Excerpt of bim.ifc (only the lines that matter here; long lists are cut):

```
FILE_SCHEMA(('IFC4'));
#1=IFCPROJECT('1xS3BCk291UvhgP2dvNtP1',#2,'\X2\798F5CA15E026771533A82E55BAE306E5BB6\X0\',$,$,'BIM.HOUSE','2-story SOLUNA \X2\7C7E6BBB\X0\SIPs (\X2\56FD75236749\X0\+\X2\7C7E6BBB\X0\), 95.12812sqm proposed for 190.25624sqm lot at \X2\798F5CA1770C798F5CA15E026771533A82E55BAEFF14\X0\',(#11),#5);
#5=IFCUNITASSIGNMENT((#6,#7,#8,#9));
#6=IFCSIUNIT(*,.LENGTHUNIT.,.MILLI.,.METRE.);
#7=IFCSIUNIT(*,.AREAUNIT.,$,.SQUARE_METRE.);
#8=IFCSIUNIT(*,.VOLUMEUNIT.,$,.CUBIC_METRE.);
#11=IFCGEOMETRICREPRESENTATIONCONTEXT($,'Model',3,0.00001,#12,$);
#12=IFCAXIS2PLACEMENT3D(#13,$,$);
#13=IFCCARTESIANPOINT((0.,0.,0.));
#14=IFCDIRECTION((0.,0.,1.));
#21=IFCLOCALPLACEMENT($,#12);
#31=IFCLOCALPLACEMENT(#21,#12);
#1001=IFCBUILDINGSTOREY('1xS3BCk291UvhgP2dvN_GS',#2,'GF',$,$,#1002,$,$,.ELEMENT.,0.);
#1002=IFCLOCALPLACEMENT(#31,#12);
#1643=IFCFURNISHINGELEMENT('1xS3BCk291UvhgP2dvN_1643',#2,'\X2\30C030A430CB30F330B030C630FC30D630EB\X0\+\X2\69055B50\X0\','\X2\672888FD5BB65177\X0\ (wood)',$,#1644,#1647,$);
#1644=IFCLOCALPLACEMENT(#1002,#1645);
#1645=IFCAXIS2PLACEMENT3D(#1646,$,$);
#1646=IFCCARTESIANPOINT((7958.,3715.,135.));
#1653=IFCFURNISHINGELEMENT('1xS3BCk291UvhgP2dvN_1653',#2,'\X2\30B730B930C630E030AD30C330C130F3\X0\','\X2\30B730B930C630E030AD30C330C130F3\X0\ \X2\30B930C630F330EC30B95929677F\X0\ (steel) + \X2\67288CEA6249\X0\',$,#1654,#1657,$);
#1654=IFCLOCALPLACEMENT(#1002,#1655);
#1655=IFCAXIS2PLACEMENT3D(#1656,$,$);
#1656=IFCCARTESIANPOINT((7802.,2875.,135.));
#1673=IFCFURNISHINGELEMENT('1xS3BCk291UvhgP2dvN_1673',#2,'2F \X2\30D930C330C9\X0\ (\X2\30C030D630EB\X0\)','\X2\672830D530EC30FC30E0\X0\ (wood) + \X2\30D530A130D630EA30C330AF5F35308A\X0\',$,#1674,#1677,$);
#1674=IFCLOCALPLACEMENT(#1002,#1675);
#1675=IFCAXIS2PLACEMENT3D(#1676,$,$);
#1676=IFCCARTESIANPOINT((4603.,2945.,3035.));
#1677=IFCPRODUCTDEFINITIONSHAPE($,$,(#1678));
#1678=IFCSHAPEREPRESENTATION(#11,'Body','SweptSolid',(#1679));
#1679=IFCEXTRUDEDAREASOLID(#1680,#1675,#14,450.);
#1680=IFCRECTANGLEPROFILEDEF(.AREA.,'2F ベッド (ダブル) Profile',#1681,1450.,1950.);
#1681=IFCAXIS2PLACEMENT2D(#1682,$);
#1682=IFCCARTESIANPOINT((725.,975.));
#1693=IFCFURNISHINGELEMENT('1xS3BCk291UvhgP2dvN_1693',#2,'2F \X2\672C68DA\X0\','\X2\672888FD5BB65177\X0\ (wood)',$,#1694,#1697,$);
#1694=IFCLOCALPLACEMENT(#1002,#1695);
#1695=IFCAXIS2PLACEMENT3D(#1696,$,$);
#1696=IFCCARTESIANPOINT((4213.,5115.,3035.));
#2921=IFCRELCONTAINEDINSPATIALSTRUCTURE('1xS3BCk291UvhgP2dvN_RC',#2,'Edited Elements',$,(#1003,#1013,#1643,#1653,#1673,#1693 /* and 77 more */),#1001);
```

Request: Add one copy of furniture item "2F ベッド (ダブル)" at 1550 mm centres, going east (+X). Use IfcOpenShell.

```python
import numpy as np
import ifcopenshell
import ifcopenshell.api.geometry
import ifcopenshell.api.root
import ifcopenshell.util.element
import ifcopenshell.util.placement
import ifcopenshell.util.unit

model = ifcopenshell.open("bim.ifc")
unit_scale = ifcopenshell.util.unit.calculate_unit_scale(model)


def reuse_history(source, copy):
    """copy_class also copies each property set's owner history, people and application; keep the originals."""
    for rel in copy.IsDefinedBy:
        if rel.is_a("IfcRelDefinesByProperties") and (history := rel.RelatingPropertyDefinition.OwnerHistory):
            rel.RelatingPropertyDefinition.OwnerHistory = source.OwnerHistory
            ifcopenshell.util.element.remove_deep2(model, history)


source = model.by_guid("1xS3BCk291UvhgP2dvN_1673")
base = ifcopenshell.util.placement.get_local_placement(source.ObjectPlacement)
step = np.array([1.0, 0.0, 0.0]) * 1.55 / unit_scale

for i in range(1, 2):
    copy = ifcopenshell.api.root.copy_class(model, product=source)
    copy.Representation = ifcopenshell.util.element.copy_deep(
        model, source.Representation, exclude=["IfcGeometricRepresentationContext", "IfcRepresentationMap"]
    )
    reuse_history(source, copy)
    matrix = base.copy()
    matrix[:3, 3] += i * step
    print("added at", matrix[:3, 3].round(3) + 0.0)
    ifcopenshell.api.geometry.edit_object_placement(model, product=copy, matrix=matrix, is_si=False)

model.write("bim-out.ifc")
```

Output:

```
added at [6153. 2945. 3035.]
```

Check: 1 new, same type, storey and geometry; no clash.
